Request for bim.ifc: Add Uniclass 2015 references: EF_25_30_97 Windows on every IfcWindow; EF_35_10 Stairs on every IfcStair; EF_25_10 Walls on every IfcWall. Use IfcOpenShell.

First a look at what the model holds.

```python
import ifcopenshell

model = ifcopenshell.open("bim.ifc")
print(model.schema)
print("classifications:", [c.Name for c in model.by_type("IfcClassification")])
for ifc_class in ("IfcDoor", "IfcRoof", "IfcStair", "IfcWall", "IfcWindow"):
    print(ifc_class, len(model.by_type(ifc_class)))
```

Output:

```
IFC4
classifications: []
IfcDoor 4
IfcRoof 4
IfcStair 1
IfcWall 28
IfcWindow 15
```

```python
import ifcopenshell
import ifcopenshell.api.classification

model = ifcopenshell.open("bim.ifc")

system = ifcopenshell.api.classification.add_classification(model, classification="Uniclass 2015")

codes = {
    "IfcWindow": ("EF_25_30_97", "Windows"),
    "IfcStair": ("EF_35_10", "Stairs"),
    "IfcWall": ("EF_25_10", "Walls"),
}
for ifc_class, (code, name) in codes.items():
    products = model.by_type(ifc_class)
    ifcopenshell.api.classification.add_reference(
        model, products=products, classification=system, identification=code, name=name
    )
    print(code, len(products))

model.write("bim_updated.ifc")
```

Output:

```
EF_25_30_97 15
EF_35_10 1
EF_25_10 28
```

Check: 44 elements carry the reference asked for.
